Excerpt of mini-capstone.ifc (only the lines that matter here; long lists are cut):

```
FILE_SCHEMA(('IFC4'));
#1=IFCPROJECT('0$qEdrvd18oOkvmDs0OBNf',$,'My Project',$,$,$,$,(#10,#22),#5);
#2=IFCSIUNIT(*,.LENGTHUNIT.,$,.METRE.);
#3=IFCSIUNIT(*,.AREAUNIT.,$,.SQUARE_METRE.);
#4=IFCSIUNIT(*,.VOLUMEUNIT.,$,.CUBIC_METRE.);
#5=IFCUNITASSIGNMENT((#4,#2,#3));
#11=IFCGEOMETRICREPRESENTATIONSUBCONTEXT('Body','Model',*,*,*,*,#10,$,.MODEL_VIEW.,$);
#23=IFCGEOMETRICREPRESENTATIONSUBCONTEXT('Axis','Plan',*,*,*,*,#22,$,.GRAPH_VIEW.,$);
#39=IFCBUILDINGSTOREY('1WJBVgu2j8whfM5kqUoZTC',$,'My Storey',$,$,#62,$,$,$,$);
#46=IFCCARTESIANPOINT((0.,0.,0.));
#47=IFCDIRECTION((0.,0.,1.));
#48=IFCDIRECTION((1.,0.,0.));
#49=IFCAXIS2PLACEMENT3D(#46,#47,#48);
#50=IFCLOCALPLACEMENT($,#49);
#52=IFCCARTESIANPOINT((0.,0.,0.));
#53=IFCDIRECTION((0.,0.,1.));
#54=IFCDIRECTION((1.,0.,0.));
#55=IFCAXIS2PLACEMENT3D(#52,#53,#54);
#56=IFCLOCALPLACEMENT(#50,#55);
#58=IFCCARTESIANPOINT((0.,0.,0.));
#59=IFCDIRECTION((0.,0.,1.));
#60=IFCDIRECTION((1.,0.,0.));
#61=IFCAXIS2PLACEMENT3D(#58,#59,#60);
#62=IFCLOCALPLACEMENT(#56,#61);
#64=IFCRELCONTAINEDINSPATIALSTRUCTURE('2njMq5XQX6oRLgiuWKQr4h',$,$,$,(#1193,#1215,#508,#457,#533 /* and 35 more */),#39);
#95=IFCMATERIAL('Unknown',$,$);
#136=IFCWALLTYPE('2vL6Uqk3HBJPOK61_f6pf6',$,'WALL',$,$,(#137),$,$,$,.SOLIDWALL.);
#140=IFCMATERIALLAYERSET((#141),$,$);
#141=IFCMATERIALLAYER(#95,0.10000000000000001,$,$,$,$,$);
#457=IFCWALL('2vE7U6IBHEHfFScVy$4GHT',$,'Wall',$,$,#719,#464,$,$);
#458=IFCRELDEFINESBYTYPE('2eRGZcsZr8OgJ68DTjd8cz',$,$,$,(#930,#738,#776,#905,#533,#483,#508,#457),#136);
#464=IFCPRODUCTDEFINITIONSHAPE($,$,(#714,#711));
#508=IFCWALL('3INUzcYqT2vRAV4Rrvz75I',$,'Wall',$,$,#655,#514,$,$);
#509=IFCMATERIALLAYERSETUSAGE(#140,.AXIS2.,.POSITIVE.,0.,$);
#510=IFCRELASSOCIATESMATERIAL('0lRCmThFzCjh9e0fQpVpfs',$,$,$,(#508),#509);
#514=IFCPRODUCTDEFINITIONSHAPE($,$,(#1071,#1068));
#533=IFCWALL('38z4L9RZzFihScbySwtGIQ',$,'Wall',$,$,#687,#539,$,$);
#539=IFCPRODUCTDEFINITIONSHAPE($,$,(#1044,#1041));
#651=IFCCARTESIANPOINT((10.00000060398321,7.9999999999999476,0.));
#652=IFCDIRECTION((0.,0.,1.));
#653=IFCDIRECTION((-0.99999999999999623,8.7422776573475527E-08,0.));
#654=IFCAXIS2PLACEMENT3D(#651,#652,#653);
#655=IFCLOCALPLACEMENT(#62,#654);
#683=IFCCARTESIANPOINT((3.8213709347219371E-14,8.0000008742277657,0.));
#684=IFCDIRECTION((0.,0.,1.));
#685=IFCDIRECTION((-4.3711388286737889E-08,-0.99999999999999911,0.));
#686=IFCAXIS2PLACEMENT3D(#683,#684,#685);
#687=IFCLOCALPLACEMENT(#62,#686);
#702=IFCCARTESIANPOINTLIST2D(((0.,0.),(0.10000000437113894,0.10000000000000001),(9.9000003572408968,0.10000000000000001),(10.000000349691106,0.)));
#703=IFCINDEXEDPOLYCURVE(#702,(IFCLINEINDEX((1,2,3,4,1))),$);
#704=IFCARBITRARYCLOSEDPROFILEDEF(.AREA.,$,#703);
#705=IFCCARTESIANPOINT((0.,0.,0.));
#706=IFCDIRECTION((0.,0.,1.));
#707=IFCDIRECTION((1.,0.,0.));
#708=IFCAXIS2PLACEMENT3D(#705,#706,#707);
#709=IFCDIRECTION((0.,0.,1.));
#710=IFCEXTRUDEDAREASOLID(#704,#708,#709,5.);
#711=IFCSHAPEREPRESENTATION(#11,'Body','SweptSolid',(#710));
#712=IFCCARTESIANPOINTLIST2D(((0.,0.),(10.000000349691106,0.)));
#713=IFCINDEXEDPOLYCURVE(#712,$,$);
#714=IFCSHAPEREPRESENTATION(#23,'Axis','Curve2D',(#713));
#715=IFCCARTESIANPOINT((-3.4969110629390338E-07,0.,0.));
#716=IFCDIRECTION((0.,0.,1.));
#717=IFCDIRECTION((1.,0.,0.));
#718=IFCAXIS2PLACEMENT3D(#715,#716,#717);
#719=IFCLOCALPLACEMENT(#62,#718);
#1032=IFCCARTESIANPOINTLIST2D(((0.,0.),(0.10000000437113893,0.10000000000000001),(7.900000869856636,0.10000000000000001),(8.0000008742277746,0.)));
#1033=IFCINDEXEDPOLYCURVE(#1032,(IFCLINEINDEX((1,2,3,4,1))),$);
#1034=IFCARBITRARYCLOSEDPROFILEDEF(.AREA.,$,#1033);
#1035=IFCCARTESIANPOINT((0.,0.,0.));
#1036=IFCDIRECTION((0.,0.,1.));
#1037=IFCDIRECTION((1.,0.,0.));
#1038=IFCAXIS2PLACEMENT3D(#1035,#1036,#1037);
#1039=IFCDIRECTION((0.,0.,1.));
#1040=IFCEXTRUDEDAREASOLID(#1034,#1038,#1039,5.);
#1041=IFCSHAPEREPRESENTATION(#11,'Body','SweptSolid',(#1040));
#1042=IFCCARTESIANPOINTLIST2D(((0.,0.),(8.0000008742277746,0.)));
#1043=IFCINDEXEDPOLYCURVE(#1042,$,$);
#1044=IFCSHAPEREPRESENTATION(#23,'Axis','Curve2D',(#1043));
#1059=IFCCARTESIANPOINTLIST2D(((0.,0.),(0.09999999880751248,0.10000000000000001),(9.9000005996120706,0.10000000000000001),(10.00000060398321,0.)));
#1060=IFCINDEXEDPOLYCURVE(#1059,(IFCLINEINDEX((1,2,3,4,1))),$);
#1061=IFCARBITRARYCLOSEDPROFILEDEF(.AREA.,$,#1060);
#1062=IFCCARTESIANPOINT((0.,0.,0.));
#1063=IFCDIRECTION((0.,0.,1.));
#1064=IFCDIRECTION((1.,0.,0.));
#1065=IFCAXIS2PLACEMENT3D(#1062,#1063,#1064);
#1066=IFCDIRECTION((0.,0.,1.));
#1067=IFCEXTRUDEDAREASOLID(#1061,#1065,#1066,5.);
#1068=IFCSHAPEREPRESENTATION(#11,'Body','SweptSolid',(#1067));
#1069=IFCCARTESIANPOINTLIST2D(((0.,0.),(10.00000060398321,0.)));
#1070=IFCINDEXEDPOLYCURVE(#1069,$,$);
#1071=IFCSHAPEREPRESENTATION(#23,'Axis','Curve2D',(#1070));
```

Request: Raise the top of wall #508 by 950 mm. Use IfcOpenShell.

```python
import ifcopenshell
import ifcopenshell.geom
import ifcopenshell.util.representation
import ifcopenshell.util.shape

model = ifcopenshell.open("mini-capstone.ifc")
settings = ifcopenshell.geom.settings()


def volume(element):
    """Net volume in cubic metres, openings subtracted."""
    shape = ifcopenshell.geom.create_shape(settings, element)
    return ifcopenshell.util.shape.get_volume(shape.geometry)


wall = model.by_guid("3INUzcYqT2vRAV4Rrvz75I")
before = volume(wall)

body = ifcopenshell.util.representation.get_representation(wall, "Model", "Body")
solid = body.Items[0]
old_height = solid.Depth
solid.Depth += 0.95
after = volume(wall)

print(f"height {old_height:g} -> {solid.Depth:g}, volume {before:.3f} -> {after:.3f} m3")

model.write("mini-capstone_rev.ifc")
```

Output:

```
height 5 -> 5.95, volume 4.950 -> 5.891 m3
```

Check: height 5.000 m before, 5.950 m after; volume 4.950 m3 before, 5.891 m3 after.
